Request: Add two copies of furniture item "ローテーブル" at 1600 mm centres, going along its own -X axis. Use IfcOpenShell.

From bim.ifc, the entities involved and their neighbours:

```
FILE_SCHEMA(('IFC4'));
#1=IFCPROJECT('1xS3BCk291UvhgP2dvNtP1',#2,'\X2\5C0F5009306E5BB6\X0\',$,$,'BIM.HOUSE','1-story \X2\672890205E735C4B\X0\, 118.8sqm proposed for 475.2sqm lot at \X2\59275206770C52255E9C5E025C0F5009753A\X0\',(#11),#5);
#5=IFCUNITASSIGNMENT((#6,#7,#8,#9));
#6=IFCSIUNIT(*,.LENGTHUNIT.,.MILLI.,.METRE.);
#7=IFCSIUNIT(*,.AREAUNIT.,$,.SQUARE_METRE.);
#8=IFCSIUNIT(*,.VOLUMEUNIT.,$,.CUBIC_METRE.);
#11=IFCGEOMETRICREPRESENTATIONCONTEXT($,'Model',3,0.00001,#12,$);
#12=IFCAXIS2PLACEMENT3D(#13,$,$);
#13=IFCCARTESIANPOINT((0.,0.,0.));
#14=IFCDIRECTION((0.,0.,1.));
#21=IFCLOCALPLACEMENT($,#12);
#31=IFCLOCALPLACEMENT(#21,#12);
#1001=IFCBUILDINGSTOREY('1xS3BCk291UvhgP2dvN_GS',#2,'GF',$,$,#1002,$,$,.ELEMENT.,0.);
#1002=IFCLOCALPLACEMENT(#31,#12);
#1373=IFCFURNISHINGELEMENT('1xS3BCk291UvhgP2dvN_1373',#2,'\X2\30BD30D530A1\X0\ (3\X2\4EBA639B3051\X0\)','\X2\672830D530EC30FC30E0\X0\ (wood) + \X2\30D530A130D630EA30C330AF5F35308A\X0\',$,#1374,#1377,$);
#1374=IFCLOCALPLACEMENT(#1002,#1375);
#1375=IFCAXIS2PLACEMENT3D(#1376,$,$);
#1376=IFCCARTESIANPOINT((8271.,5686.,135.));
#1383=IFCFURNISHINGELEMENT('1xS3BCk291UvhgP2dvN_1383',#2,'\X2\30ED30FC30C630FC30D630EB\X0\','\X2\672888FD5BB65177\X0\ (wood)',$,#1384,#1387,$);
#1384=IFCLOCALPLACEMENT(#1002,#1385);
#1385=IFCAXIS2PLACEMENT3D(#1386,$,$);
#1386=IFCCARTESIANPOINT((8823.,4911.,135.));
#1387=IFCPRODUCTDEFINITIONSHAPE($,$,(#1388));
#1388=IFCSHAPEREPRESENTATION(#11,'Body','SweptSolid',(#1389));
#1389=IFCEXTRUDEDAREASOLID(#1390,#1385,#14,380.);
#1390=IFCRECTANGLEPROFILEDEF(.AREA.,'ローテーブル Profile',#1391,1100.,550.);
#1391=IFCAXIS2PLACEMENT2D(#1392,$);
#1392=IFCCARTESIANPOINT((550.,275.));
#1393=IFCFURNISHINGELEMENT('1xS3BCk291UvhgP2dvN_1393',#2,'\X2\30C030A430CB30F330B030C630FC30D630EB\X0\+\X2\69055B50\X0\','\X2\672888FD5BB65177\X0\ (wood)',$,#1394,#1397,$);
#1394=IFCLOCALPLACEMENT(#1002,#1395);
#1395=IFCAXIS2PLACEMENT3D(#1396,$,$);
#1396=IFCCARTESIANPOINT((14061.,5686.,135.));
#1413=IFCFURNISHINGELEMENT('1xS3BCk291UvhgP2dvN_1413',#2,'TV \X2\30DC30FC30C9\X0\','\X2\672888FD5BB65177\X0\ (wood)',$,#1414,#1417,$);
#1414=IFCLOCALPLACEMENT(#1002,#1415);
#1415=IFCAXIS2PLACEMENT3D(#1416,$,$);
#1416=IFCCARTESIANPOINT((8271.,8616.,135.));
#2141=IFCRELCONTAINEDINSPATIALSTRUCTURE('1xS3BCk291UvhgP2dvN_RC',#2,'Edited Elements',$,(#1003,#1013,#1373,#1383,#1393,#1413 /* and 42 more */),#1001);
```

```python
import ifcopenshell
import ifcopenshell.api.geometry
import ifcopenshell.api.root
import ifcopenshell.util.element
import ifcopenshell.util.placement
import ifcopenshell.util.unit

model = ifcopenshell.open("bim.ifc")
unit_scale = ifcopenshell.util.unit.calculate_unit_scale(model)


def reuse_history(source, copy):
    """copy_class also copies each property set's owner history, people and application; keep the originals."""
    for rel in copy.IsDefinedBy:
        if rel.is_a("IfcRelDefinesByProperties") and (history := rel.RelatingPropertyDefinition.OwnerHistory):
            rel.RelatingPropertyDefinition.OwnerHistory = source.OwnerHistory
            ifcopenshell.util.element.remove_deep2(model, history)


source = model.by_id(1383)
base = ifcopenshell.util.placement.get_local_placement(source.ObjectPlacement)
step = -base[:3, 0] * 1.6 / unit_scale

for i in range(1, 3):
    copy = ifcopenshell.api.root.copy_class(model, product=source)
    copy.Representation = ifcopenshell.util.element.copy_deep(
        model, source.Representation, exclude=["IfcGeometricRepresentationContext", "IfcRepresentationMap"]
    )
    reuse_history(source, copy)
    matrix = base.copy()
    matrix[:3, 3] += i * step
    print("added at", matrix[:3, 3].round(3) + 0.0)
    ifcopenshell.api.geometry.edit_object_placement(model, product=copy, matrix=matrix, is_si=False)

model.write("bim_edited.ifc")
```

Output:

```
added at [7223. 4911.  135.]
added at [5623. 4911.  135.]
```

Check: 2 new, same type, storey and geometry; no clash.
